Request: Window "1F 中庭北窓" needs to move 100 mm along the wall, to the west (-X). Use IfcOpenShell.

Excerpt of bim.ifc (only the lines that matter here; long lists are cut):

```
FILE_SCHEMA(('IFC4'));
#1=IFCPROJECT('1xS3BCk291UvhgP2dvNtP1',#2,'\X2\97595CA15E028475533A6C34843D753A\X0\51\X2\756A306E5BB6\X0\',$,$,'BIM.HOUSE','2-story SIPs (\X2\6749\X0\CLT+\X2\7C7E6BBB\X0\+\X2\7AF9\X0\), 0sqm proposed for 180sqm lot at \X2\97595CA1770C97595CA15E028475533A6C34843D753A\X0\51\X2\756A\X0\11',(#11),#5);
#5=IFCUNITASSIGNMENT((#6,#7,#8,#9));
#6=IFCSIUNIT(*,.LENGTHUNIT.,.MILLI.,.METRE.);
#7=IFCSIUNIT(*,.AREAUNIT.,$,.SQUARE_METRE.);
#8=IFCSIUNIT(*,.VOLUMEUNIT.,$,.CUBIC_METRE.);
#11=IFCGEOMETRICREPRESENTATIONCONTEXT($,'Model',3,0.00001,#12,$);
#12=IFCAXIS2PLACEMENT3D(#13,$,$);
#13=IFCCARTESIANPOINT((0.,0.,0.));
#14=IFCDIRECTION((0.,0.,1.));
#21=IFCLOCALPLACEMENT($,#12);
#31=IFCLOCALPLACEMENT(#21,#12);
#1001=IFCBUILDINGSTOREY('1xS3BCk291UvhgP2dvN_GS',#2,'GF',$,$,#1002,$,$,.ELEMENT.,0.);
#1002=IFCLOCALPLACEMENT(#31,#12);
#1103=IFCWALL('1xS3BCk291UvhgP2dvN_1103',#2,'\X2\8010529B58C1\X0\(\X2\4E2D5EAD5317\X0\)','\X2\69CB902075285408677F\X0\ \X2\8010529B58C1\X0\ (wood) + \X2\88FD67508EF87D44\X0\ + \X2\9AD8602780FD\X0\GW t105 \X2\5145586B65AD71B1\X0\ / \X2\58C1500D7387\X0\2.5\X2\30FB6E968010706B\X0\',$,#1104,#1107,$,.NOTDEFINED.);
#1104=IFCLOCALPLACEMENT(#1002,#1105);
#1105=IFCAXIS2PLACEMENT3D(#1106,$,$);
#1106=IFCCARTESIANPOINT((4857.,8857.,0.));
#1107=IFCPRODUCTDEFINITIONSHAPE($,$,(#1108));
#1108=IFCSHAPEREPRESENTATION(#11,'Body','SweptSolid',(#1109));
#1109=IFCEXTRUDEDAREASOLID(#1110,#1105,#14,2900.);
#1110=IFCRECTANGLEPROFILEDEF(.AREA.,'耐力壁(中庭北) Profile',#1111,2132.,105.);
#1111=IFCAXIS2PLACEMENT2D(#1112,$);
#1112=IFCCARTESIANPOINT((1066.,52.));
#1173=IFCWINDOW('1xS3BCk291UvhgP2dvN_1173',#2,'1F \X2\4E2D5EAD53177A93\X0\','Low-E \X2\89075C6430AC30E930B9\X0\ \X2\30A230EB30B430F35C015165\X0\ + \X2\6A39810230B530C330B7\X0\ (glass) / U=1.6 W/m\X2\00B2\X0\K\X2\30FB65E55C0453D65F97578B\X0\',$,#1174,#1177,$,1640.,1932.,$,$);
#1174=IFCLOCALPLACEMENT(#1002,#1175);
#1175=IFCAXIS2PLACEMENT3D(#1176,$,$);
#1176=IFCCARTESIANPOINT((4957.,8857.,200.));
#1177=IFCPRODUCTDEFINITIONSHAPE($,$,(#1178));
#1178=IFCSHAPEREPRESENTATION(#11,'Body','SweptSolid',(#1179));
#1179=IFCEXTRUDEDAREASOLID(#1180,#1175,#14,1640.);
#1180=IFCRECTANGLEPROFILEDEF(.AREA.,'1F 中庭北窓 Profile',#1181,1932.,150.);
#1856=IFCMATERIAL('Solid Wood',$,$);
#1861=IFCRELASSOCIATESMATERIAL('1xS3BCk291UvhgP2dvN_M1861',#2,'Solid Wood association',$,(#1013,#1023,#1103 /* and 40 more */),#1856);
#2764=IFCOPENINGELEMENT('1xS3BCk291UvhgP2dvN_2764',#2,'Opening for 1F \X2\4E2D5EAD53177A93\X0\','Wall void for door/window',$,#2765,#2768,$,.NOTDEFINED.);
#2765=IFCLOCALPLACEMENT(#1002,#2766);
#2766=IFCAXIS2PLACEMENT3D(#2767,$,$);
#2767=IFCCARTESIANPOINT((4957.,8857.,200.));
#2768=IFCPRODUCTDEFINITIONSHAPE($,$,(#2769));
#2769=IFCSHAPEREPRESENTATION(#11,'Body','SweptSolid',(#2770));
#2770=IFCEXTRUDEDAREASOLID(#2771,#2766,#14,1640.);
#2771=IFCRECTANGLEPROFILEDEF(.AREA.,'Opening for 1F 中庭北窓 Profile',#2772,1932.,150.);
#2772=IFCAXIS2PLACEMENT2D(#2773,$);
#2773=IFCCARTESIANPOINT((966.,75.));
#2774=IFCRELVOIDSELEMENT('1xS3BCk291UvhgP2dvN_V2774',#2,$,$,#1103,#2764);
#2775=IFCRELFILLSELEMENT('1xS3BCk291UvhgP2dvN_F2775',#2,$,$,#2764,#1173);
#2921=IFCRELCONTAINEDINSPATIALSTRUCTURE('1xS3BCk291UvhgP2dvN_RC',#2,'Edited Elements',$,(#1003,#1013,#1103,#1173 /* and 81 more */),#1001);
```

```python
import ifcopenshell
import ifcopenshell.api.geometry
import ifcopenshell.util.placement
import ifcopenshell.util.unit

model = ifcopenshell.open("bim.ifc")
unit_scale = ifcopenshell.util.unit.calculate_unit_scale(model)

window = model.by_guid("1xS3BCk291UvhgP2dvN_1173")
opening = window.FillsVoids[0].RelatingOpeningElement
wall = opening.VoidsElements[0].RelatingBuildingElement

wall_matrix = ifcopenshell.util.placement.get_local_placement(wall.ObjectPlacement)
shift = wall_matrix[:3, 0] * -0.1 / unit_scale
before = ifcopenshell.util.placement.get_local_placement(window.ObjectPlacement)[:3, 3].copy()

# The window is not placed relative to its opening, so move both.
for product in (opening, window):
    matrix = ifcopenshell.util.placement.get_local_placement(product.ObjectPlacement)
    matrix[:3, 3] += shift
    ifcopenshell.api.geometry.edit_object_placement(model, product=product, matrix=matrix, is_si=False)

after = ifcopenshell.util.placement.get_local_placement(window.ObjectPlacement)[:3, 3]
print("window moved by", (after - before).round(3) + 0.0)

model.write("bim_rev.ifc")
```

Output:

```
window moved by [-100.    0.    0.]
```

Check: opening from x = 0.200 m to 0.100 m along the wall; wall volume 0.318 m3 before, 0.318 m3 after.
